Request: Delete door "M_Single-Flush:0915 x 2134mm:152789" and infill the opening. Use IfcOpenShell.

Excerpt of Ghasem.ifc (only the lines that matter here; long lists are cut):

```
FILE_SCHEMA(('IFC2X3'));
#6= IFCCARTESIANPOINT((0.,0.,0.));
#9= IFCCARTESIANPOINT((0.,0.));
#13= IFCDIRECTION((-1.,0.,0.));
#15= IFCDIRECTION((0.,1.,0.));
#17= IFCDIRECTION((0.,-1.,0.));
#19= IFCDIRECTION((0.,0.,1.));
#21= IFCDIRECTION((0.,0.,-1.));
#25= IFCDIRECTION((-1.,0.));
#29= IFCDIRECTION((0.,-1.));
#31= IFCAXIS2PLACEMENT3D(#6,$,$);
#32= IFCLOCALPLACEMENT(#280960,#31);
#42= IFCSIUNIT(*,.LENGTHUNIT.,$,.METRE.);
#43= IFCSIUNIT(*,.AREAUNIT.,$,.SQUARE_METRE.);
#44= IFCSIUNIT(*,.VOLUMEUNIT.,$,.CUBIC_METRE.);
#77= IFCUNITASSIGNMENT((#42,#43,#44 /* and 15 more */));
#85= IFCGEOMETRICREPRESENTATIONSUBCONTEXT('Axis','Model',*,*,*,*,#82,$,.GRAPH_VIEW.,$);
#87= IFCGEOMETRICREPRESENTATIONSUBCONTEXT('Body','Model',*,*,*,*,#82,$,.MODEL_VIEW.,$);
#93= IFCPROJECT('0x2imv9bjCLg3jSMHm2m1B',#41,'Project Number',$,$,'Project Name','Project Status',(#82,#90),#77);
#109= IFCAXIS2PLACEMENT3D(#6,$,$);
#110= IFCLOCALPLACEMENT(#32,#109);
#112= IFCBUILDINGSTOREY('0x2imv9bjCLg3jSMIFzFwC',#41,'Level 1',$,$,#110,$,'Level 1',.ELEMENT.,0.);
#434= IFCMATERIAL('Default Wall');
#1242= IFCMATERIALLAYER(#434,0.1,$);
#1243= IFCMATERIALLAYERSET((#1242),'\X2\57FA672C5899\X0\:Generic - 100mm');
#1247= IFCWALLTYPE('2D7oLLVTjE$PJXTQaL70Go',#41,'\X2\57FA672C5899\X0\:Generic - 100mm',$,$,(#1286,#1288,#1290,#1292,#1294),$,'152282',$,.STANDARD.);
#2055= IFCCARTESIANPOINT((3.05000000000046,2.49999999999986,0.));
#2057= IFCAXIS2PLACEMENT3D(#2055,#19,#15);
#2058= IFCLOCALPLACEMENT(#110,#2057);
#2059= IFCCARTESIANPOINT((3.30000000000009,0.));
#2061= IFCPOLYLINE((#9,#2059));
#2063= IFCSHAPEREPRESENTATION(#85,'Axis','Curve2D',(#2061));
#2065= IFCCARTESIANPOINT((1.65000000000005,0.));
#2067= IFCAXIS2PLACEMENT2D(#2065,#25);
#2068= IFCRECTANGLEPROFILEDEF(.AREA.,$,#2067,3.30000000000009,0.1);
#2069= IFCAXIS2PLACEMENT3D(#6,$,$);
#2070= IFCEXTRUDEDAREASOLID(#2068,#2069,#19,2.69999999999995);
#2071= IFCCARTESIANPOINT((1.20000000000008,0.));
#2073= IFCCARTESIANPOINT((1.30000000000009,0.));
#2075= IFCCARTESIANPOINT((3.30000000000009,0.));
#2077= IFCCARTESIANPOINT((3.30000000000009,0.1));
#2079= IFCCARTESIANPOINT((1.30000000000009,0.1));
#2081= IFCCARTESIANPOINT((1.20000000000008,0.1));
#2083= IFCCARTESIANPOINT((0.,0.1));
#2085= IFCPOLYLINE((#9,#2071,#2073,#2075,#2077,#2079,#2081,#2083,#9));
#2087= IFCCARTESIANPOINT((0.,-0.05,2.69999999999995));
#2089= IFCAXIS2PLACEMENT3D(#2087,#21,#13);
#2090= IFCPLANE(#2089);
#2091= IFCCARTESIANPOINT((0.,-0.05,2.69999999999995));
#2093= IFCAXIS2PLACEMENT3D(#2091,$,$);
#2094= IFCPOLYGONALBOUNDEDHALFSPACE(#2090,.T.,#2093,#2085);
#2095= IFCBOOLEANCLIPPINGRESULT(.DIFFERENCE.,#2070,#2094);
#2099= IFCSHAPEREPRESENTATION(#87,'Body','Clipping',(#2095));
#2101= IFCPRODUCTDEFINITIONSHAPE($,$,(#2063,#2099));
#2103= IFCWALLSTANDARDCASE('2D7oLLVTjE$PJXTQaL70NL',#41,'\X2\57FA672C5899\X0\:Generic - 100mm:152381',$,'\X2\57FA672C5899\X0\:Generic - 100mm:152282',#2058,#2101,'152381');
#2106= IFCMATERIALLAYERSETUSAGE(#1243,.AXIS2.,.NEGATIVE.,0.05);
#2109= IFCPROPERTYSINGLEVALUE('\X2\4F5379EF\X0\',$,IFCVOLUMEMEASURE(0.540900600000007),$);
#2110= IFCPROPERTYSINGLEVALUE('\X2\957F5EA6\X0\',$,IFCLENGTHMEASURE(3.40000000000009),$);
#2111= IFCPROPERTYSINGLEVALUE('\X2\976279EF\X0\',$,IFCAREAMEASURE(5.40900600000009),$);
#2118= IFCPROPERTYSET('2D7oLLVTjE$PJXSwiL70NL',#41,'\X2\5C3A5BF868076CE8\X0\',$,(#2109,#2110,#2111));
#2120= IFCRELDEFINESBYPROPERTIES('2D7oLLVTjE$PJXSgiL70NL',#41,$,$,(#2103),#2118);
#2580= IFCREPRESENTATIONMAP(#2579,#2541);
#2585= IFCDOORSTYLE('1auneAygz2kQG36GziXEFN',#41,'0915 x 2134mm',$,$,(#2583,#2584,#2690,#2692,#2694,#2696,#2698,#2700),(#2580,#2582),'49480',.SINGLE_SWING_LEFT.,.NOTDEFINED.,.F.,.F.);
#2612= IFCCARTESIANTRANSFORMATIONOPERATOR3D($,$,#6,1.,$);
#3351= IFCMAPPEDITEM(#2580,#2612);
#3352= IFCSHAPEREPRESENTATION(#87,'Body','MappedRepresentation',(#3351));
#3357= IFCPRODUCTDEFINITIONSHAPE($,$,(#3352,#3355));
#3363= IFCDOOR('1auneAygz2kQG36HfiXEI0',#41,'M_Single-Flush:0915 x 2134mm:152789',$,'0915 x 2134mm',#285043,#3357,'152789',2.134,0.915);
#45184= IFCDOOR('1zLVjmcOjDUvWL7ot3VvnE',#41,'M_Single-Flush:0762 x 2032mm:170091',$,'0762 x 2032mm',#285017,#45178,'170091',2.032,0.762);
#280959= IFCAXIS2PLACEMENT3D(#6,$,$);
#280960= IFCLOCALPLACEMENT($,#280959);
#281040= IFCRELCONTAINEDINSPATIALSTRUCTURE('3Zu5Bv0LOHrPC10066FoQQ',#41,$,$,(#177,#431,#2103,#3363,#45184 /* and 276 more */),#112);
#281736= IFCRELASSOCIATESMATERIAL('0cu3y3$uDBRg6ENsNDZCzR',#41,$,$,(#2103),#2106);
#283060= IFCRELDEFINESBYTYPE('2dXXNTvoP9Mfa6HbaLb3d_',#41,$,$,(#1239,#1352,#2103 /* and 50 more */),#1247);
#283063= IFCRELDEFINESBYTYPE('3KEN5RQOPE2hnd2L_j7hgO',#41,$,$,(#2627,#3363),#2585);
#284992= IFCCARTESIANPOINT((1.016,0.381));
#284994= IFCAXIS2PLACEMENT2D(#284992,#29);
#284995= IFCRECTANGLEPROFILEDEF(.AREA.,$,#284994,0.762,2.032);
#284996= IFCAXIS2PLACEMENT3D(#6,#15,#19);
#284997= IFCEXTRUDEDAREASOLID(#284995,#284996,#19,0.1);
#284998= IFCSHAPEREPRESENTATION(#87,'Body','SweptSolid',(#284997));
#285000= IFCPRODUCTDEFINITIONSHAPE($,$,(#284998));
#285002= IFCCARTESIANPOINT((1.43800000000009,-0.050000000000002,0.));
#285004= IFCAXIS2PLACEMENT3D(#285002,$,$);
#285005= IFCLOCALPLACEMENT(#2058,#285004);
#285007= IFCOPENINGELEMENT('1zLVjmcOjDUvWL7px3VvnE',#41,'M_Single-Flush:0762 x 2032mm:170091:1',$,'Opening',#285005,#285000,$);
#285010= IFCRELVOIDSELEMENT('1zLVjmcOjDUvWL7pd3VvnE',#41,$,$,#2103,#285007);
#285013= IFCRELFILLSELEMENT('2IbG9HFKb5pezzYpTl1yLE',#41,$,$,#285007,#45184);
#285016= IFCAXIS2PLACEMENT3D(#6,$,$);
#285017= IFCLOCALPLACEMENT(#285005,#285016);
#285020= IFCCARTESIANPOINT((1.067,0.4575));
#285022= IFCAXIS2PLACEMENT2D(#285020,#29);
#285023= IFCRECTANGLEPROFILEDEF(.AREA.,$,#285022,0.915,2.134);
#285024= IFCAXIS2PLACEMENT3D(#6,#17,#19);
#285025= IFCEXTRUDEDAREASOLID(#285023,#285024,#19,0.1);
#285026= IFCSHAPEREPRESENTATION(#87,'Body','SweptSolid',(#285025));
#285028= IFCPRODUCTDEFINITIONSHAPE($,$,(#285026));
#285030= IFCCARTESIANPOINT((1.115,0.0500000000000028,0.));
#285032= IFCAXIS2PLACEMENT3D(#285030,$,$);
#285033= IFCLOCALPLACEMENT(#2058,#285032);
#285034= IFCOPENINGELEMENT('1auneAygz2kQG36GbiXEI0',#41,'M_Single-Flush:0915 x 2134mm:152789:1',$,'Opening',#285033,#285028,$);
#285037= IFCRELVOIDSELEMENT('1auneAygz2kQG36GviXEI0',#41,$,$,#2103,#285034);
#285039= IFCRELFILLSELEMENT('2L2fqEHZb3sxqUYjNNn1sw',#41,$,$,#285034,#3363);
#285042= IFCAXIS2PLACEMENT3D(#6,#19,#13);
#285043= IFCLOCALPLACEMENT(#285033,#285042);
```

```python
import ifcopenshell
import ifcopenshell.api.feature
import ifcopenshell.api.pset
import ifcopenshell.api.root
import ifcopenshell.geom
import ifcopenshell.util.element
import ifcopenshell.util.shape
import ifcopenshell.util.unit

model = ifcopenshell.open("Ghasem.ifc")
area_scale = ifcopenshell.util.unit.calculate_unit_scale(model, "AREAUNIT")
volume_scale = ifcopenshell.util.unit.calculate_unit_scale(model, "VOLUMEUNIT")
settings = ifcopenshell.geom.settings()


def volume(element):
    """Net volume in cubic metres, openings subtracted."""
    shape = ifcopenshell.geom.create_shape(settings, element)
    return ifcopenshell.util.shape.get_volume(shape.geometry)


door = model.by_id(3363)
opening = door.FillsVoids[0].RelatingOpeningElement
wall = opening.VoidsElements[0].RelatingBuildingElement
before = volume(wall)

ifcopenshell.api.root.remove_product(model, product=door)
ifcopenshell.api.feature.remove_feature(model, feature=opening)

after = volume(wall)
thickness = 0.1  # wall thickness in metres

# Update the wall's stored quantities.
pset = model.by_id(ifcopenshell.util.element.get_pset(wall, "尺寸标注", should_inherit=False)["id"])
ifcopenshell.api.pset.edit_pset(model, pset=pset, properties={
    "体积": model.create_entity("IfcVolumeMeasure", after / volume_scale),
    "面积": model.create_entity("IfcAreaMeasure", after / thickness / area_scale),
})

print(f"wall volume {before:.3f} -> {after:.3f} m3")

model.write("Ghasem_edited.ifc")
```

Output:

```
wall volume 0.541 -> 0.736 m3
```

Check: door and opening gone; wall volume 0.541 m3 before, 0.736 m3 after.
